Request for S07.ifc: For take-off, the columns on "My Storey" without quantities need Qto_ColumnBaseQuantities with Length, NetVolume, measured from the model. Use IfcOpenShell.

First a look at what the model holds.

```python
import ifcopenshell
import ifcopenshell.util.element
import ifcopenshell.util.unit

model = ifcopenshell.open("S07.ifc")
print(model.schema)
for unit_type in ("LENGTHUNIT", "AREAUNIT", "VOLUMEUNIT"):
    print(unit_type, ifcopenshell.util.unit.calculate_unit_scale(model, unit_type))
storey = next(s for s in model.by_type("IfcBuildingStorey") if s.Name == "My Storey")
columns = [e for e in ifcopenshell.util.element.get_decomposition(storey) if e.is_a("IfcColumn")]
for e in sorted(columns, key=lambda e: e.id()):
    print(e.id(), e.is_a(), e.Name, list(ifcopenshell.util.element.get_psets(e, qtos_only=True)), sep=" | ")
```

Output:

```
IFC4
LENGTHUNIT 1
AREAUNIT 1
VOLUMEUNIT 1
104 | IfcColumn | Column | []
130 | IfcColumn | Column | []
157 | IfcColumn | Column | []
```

```python
import ifcopenshell
import ifcopenshell.api.pset
import ifcopenshell.geom
import ifcopenshell.util.element
import ifcopenshell.util.shape
import ifcopenshell.util.unit

model = ifcopenshell.open("S07.ifc")
unit_scale = ifcopenshell.util.unit.calculate_unit_scale(model)
volume_scale = ifcopenshell.util.unit.calculate_unit_scale(model, "VOLUMEUNIT")
settings = ifcopenshell.geom.settings()

storey = next(s for s in model.by_type("IfcBuildingStorey") if s.Name == "My Storey")
columns = [e for e in ifcopenshell.util.element.get_decomposition(storey) if e.is_a("IfcColumn")]

for e in sorted(columns, key=lambda e: e.id()):
    if ifcopenshell.util.element.get_psets(e, qtos_only=True, should_inherit=False):
        continue
    # Geometry comes back in metres, in the element's own axes.
    shape = ifcopenshell.geom.create_shape(settings, e)
    values = {
        "Length": ifcopenshell.util.shape.get_z(shape.geometry) / unit_scale,
        "NetVolume": ifcopenshell.util.shape.get_volume(shape.geometry) / volume_scale,
    }
    qto = ifcopenshell.api.pset.add_qto(model, product=e, name="Qto_ColumnBaseQuantities")
    ifcopenshell.api.pset.edit_qto(model, qto=qto, properties=values)
    print(e.id(), {k: round(v, 3) for k, v in values.items()})

model.write("S07_edited.ifc")
```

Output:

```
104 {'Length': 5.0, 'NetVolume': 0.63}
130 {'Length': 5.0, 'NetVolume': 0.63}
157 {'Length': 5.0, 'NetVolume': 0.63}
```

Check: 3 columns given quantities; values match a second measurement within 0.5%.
